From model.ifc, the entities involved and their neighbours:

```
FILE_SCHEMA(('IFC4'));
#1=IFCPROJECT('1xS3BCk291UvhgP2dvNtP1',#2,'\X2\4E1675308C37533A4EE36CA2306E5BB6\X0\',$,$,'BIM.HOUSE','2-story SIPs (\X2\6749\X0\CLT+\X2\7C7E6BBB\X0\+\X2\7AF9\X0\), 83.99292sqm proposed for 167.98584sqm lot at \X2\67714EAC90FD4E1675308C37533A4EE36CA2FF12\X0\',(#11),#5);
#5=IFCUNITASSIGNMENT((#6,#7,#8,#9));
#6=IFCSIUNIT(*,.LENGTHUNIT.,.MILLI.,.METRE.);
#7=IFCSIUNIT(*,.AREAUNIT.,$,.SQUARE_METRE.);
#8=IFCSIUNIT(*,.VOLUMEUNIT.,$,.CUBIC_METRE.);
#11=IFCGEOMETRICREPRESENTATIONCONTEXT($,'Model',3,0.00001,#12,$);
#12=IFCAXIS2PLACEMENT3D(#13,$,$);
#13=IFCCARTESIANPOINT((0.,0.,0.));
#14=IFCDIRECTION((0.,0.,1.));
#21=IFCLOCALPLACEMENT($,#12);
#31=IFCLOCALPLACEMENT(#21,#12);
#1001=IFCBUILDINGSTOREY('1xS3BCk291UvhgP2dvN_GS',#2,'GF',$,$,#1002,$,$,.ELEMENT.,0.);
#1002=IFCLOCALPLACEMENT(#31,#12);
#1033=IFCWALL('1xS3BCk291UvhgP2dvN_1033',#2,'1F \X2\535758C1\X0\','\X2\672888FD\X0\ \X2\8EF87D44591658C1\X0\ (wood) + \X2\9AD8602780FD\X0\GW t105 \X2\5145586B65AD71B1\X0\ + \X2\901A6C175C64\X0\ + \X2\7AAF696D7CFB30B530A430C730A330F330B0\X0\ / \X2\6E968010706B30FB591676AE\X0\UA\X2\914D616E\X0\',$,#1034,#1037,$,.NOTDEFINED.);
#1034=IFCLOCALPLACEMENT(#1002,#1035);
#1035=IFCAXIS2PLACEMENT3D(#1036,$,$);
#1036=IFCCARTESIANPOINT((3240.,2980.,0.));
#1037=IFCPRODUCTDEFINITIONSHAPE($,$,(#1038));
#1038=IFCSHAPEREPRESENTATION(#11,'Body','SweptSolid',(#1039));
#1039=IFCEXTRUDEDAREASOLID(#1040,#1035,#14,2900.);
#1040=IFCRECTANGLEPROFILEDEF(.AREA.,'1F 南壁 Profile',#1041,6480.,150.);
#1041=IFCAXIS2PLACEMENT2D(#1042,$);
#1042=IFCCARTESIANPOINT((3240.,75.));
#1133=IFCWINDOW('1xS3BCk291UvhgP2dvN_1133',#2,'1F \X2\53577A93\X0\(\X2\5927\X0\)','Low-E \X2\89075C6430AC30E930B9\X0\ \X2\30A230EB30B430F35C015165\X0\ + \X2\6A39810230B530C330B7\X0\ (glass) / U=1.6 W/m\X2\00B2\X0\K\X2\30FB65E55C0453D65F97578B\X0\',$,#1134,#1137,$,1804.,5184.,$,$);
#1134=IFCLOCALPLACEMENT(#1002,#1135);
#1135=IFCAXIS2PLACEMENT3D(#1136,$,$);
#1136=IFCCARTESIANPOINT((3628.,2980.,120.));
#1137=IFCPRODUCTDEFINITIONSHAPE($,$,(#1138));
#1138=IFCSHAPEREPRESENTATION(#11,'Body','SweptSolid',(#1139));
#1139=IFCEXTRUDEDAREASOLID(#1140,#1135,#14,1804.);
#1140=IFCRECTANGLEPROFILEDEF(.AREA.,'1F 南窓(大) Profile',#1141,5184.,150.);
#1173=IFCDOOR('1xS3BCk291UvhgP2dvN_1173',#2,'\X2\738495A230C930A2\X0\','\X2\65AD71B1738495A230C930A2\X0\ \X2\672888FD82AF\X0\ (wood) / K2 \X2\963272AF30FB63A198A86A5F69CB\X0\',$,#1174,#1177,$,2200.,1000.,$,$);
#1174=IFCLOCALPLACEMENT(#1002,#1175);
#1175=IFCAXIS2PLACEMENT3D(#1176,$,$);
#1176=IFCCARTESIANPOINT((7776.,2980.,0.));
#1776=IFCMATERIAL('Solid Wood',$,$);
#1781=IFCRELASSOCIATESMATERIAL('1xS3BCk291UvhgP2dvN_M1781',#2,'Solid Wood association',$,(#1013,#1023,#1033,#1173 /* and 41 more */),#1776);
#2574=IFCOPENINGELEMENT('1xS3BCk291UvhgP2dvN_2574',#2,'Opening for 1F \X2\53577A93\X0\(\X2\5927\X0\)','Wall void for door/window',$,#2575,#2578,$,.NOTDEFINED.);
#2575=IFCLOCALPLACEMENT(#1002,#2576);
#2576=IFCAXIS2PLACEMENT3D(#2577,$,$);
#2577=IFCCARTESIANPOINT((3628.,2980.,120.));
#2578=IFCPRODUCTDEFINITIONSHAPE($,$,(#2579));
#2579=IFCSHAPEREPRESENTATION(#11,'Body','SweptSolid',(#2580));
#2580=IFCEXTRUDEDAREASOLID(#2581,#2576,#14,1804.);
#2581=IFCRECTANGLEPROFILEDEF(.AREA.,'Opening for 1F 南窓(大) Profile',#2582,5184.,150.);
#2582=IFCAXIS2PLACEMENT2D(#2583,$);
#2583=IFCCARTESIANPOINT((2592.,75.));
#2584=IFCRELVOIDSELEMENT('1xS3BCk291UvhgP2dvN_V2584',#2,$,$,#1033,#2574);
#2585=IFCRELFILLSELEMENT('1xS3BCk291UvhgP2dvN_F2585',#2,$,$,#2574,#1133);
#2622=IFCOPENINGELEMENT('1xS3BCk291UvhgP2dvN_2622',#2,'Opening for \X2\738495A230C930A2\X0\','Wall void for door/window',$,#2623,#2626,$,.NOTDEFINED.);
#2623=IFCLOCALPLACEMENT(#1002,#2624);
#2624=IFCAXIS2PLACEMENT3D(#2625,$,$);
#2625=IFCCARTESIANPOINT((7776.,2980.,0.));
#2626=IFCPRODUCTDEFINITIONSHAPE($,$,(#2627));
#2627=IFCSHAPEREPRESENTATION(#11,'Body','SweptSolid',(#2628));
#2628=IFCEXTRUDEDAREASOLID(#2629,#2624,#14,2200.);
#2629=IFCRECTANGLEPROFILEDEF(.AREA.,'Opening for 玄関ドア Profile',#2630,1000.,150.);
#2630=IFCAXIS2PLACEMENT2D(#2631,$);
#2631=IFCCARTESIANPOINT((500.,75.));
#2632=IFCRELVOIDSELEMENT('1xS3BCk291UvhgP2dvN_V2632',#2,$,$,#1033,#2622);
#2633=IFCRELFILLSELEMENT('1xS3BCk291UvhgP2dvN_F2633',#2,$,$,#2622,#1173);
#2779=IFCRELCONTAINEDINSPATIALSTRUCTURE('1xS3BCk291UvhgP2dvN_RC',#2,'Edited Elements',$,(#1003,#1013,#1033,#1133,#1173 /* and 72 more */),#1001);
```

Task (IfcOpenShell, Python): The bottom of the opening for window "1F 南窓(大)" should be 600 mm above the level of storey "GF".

```python
import numpy as np
import ifcopenshell
import ifcopenshell.api.geometry
import ifcopenshell.geom
import ifcopenshell.util.element
import ifcopenshell.util.placement
import ifcopenshell.util.shape
import ifcopenshell.util.unit

model = ifcopenshell.open("model.ifc")
unit_scale = ifcopenshell.util.unit.calculate_unit_scale(model)

window = model.by_guid("1xS3BCk291UvhgP2dvN_1133")
opening = window.FillsVoids[0].RelatingOpeningElement
storey = ifcopenshell.util.element.get_container(window, ifc_class="IfcBuildingStorey")
level = ifcopenshell.util.placement.get_local_placement(storey.ObjectPlacement)[2, 3]

# The opening's origin need not be at the sill, so measure its lowest point.
shape = ifcopenshell.geom.create_shape(ifcopenshell.geom.settings(), opening)
bottom = ifcopenshell.util.shape.get_shape_bottom_elevation(shape, shape.geometry) / unit_scale
dz = level + 600.0 - bottom

shift = np.array([0.0, 0.0, dz])
# The window is not placed relative to its opening, so move both.
for product in (opening, window):
    matrix = ifcopenshell.util.placement.get_local_placement(product.ObjectPlacement)
    matrix[:3, 3] += shift
    ifcopenshell.api.geometry.edit_object_placement(model, product=product, matrix=matrix, is_si=False)

print(f"moved by {dz * unit_scale:+.3f} m")

model.write("model-out.ifc")
```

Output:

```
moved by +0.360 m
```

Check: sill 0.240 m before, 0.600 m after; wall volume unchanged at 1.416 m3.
